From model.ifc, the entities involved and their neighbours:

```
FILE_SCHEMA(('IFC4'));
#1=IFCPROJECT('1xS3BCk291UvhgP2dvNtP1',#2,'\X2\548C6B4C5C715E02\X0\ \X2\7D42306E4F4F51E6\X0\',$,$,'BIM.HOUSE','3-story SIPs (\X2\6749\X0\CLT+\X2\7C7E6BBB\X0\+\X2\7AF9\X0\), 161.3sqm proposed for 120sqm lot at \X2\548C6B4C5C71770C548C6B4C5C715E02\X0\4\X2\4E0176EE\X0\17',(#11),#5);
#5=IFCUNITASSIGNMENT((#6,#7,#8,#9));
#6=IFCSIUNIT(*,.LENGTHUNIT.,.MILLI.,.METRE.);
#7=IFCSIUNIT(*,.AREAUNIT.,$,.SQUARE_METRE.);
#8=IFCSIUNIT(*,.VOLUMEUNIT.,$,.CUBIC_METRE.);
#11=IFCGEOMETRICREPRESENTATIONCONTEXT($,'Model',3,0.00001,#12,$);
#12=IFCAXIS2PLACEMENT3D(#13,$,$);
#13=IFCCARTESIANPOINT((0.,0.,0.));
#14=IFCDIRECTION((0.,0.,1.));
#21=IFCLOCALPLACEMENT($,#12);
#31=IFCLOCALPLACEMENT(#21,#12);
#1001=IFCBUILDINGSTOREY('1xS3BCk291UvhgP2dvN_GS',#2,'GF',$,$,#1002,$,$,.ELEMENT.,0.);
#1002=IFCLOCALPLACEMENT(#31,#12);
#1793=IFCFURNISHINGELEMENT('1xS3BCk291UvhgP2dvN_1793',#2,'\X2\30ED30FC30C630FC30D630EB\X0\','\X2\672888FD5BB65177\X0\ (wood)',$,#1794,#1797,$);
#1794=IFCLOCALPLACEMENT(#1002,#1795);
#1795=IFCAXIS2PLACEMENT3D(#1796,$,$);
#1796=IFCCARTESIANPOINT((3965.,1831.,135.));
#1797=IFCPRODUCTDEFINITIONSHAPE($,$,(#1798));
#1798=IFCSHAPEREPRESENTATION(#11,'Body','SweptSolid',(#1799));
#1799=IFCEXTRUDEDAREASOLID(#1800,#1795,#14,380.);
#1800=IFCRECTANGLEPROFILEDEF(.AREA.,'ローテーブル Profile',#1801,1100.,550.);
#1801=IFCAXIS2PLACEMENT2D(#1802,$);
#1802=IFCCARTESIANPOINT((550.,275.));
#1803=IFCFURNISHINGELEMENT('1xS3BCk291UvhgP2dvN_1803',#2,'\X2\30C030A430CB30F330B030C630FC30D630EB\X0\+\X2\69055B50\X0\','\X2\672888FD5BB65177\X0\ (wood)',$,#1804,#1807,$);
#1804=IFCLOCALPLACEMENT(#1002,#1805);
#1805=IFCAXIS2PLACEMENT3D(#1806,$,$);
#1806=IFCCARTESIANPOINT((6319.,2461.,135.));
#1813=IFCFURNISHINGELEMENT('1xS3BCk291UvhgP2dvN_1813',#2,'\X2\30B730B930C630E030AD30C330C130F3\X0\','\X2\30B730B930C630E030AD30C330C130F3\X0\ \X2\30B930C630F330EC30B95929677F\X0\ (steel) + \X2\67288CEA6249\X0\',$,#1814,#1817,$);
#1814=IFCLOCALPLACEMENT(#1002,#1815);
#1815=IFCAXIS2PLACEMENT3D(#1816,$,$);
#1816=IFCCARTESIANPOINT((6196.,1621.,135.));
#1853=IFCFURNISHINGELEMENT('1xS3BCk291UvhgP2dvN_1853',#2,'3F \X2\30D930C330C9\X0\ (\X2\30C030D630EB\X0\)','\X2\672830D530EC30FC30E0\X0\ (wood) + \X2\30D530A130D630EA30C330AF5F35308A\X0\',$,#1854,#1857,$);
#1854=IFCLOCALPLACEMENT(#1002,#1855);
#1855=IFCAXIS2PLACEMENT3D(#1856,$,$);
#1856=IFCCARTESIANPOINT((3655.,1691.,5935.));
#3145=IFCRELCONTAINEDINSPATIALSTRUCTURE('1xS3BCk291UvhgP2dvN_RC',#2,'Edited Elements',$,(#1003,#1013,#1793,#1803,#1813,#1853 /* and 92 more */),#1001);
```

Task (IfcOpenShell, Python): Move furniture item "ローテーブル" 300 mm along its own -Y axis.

```python
import ifcopenshell
import ifcopenshell.api.geometry
import ifcopenshell.util.placement

model = ifcopenshell.open("model.ifc")

item = model.by_id(1793)
matrix = ifcopenshell.util.placement.get_local_placement(item.ObjectPlacement)
matrix[:3, 3] -= matrix[:3, 1] * 300.0
ifcopenshell.api.geometry.edit_object_placement(model, product=item, matrix=matrix, is_si=False)

print(ifcopenshell.util.placement.get_local_placement(item.ObjectPlacement).round(3) + 0.0)

model.write("model_v2.ifc")
```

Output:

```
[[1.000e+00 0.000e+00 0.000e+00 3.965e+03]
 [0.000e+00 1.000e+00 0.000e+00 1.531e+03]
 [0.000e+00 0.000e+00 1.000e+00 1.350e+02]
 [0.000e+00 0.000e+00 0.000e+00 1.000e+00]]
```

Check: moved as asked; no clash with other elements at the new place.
